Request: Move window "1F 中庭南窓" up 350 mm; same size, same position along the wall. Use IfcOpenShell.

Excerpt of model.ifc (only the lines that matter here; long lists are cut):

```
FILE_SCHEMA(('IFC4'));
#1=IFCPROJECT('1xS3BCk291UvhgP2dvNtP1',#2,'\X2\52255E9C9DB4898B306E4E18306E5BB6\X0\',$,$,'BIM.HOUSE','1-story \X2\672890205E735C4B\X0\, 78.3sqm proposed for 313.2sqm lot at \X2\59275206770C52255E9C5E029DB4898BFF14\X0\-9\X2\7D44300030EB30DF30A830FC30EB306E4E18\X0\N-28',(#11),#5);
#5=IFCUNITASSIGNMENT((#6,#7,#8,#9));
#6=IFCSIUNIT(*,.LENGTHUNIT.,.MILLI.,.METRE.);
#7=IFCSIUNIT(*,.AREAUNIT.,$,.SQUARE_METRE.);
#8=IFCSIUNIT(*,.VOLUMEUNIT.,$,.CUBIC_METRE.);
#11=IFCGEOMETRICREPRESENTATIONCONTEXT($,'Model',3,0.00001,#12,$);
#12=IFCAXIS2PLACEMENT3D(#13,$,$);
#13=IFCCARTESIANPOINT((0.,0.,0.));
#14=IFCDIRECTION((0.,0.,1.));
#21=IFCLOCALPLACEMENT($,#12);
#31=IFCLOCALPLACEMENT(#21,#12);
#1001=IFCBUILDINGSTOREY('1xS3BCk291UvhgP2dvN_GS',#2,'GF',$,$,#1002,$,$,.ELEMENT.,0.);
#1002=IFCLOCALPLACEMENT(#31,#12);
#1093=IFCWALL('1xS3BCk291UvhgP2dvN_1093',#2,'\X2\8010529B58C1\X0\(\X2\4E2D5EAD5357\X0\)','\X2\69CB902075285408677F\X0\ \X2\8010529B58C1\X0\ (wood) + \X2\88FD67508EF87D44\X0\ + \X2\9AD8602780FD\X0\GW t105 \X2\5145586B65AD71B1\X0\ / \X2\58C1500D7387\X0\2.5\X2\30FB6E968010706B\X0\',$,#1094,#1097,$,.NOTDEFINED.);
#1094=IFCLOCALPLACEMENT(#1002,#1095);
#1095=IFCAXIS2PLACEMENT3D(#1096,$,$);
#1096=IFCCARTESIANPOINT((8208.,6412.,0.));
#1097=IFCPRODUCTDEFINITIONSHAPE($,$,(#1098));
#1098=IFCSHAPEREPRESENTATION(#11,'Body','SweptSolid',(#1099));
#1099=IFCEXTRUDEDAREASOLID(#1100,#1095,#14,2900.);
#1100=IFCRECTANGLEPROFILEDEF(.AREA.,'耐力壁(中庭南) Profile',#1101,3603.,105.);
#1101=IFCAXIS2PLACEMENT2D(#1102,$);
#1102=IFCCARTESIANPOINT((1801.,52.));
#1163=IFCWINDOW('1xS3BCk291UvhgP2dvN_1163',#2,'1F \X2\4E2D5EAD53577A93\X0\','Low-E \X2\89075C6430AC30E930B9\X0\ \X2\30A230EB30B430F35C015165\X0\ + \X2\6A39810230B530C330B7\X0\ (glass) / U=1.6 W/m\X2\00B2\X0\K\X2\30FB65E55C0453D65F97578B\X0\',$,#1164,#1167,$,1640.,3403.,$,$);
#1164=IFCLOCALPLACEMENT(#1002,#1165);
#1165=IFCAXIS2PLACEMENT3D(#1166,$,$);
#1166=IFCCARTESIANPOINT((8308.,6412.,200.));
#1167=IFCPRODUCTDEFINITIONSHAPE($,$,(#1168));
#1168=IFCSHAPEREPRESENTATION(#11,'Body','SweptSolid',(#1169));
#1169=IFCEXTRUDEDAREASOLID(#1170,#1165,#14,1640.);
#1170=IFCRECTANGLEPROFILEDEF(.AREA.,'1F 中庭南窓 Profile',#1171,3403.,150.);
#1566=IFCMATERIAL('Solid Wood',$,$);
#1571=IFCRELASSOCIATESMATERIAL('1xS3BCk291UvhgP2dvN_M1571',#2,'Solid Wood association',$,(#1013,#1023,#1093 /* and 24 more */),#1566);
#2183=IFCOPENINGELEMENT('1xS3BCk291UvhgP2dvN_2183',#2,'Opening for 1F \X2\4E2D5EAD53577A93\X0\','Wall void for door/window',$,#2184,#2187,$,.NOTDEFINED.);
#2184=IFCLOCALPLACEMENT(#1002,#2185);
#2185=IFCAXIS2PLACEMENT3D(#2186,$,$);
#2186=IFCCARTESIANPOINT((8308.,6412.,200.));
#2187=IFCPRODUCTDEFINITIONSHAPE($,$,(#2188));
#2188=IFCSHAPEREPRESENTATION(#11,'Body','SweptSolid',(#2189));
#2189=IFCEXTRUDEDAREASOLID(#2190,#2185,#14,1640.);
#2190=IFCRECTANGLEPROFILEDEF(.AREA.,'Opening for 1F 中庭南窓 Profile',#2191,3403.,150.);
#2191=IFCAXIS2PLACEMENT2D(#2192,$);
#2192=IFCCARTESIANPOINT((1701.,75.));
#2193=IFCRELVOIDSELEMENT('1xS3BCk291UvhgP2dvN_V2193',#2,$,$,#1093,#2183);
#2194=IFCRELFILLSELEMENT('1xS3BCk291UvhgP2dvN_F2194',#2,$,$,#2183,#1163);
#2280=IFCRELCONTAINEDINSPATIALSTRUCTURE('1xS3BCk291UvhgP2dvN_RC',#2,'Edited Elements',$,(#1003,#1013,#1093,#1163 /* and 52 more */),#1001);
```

```python
import numpy as np
import ifcopenshell
import ifcopenshell.api.geometry
import ifcopenshell.util.placement
import ifcopenshell.util.unit

model = ifcopenshell.open("model.ifc")
unit_scale = ifcopenshell.util.unit.calculate_unit_scale(model)

window = model.by_guid("1xS3BCk291UvhgP2dvN_1163")
opening = window.FillsVoids[0].RelatingOpeningElement
dz = 0.35 / unit_scale

shift = np.array([0.0, 0.0, dz])
# The window is not placed relative to its opening, so move both.
for product in (opening, window):
    matrix = ifcopenshell.util.placement.get_local_placement(product.ObjectPlacement)
    matrix[:3, 3] += shift
    ifcopenshell.api.geometry.edit_object_placement(model, product=product, matrix=matrix, is_si=False)

print(f"moved by {dz * unit_scale:+.3f} m")

model.write("model-out.ifc")
```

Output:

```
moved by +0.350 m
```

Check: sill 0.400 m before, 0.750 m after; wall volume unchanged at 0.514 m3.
